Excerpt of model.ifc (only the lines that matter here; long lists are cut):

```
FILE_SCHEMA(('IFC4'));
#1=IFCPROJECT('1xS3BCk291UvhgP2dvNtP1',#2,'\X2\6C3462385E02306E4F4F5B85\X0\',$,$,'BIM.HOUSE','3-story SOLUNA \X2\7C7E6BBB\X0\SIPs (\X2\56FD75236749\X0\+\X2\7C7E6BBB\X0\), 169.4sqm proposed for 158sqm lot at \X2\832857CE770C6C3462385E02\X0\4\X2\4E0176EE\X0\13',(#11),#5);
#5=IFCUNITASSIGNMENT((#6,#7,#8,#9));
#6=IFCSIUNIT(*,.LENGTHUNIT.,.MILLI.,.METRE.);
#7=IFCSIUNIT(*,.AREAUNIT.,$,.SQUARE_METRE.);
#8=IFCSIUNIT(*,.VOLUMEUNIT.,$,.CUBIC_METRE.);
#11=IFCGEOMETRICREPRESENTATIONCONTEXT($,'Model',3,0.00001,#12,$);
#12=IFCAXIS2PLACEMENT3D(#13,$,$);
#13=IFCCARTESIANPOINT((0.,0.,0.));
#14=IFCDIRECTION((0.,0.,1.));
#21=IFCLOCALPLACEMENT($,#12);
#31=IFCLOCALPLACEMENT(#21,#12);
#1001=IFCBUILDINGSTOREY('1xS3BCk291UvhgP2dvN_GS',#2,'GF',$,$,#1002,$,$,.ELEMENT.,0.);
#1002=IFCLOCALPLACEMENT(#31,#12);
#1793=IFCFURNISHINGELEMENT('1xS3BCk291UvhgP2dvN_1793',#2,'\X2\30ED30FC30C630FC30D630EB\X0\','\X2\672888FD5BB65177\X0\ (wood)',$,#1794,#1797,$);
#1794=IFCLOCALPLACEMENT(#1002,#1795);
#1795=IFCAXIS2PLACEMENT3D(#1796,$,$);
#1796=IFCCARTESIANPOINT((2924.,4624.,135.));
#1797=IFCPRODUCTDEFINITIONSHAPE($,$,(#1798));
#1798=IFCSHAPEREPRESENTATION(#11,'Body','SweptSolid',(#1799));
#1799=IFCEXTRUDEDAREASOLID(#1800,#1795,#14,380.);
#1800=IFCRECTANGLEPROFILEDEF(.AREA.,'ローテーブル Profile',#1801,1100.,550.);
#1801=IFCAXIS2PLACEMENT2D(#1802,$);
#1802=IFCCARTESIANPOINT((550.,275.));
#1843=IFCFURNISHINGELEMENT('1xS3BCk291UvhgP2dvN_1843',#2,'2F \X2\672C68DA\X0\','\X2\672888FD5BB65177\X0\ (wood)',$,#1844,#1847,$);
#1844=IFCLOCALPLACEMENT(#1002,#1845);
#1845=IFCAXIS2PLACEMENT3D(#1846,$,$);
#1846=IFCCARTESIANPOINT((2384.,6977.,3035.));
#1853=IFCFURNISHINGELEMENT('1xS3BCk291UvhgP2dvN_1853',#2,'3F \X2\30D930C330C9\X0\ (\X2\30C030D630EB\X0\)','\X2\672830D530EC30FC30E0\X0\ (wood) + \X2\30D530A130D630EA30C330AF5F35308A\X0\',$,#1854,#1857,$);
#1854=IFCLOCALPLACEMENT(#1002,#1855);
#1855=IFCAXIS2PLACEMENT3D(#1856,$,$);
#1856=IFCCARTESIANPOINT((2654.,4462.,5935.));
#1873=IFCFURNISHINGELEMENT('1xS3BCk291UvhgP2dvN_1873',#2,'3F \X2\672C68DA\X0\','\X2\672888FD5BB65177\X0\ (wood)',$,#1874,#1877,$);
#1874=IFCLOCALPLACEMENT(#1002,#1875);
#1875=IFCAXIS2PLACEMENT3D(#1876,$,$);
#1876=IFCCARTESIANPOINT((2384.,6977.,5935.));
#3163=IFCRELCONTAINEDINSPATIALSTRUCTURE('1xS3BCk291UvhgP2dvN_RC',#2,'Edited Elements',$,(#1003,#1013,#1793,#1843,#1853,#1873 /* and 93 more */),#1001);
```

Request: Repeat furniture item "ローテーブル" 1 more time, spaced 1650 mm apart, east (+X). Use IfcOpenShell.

```python
import numpy as np
import ifcopenshell
import ifcopenshell.api.geometry
import ifcopenshell.api.root
import ifcopenshell.util.element
import ifcopenshell.util.placement
import ifcopenshell.util.unit

model = ifcopenshell.open("model.ifc")
unit_scale = ifcopenshell.util.unit.calculate_unit_scale(model)


def reuse_history(source, copy):
    """copy_class also copies each property set's owner history, people and application; keep the originals."""
    for rel in copy.IsDefinedBy:
        if rel.is_a("IfcRelDefinesByProperties") and (history := rel.RelatingPropertyDefinition.OwnerHistory):
            rel.RelatingPropertyDefinition.OwnerHistory = source.OwnerHistory
            ifcopenshell.util.element.remove_deep2(model, history)


source = model.by_guid("1xS3BCk291UvhgP2dvN_1793")
base = ifcopenshell.util.placement.get_local_placement(source.ObjectPlacement)
step = np.array([1.0, 0.0, 0.0]) * 1.65 / unit_scale

for i in range(1, 2):
    copy = ifcopenshell.api.root.copy_class(model, product=source)
    copy.Representation = ifcopenshell.util.element.copy_deep(
        model, source.Representation, exclude=["IfcGeometricRepresentationContext", "IfcRepresentationMap"]
    )
    reuse_history(source, copy)
    matrix = base.copy()
    matrix[:3, 3] += i * step
    print("added at", matrix[:3, 3].round(3) + 0.0)
    ifcopenshell.api.geometry.edit_object_placement(model, product=copy, matrix=matrix, is_si=False)

model.write("model_v2.ifc")
```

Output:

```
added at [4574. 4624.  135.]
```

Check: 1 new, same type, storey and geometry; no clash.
